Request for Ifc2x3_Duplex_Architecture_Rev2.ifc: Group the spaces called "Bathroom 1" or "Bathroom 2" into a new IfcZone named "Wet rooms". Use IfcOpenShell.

First a look at what the model holds.

```python
import ifcopenshell

model = ifcopenshell.open("Ifc2x3_Duplex_Architecture_Rev2.ifc")
print(model.schema)
seen = {}
for space in model.by_type("IfcSpace"):
    seen[space.LongName] = seen.get(space.LongName, 0) + 1
for name, count in sorted(seen.items(), key=str):
    print(count, "x", name)
print("zones:", [z.Name for z in model.by_type("IfcZone")][:20])
```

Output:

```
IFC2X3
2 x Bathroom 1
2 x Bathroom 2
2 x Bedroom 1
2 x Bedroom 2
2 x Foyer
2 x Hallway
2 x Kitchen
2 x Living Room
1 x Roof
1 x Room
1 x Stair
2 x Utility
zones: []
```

```python
import ifcopenshell
import ifcopenshell.api.group
import ifcopenshell.api.root

model = ifcopenshell.open("Ifc2x3_Duplex_Architecture_Rev2.ifc")

names = {"Bathroom 1", "Bathroom 2"}
spaces = [s for s in model.by_type("IfcSpace") if s.LongName in names]

zone = ifcopenshell.api.root.create_entity(model, ifc_class="IfcZone", name="Wet rooms")
ifcopenshell.api.group.assign_group(model, products=spaces, group=zone)
print(len(spaces), "spaces in", zone.Name)

model.write("Ifc2x3_Duplex_Architecture_Rev2_edited.ifc")
```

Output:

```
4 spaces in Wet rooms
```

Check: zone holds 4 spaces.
